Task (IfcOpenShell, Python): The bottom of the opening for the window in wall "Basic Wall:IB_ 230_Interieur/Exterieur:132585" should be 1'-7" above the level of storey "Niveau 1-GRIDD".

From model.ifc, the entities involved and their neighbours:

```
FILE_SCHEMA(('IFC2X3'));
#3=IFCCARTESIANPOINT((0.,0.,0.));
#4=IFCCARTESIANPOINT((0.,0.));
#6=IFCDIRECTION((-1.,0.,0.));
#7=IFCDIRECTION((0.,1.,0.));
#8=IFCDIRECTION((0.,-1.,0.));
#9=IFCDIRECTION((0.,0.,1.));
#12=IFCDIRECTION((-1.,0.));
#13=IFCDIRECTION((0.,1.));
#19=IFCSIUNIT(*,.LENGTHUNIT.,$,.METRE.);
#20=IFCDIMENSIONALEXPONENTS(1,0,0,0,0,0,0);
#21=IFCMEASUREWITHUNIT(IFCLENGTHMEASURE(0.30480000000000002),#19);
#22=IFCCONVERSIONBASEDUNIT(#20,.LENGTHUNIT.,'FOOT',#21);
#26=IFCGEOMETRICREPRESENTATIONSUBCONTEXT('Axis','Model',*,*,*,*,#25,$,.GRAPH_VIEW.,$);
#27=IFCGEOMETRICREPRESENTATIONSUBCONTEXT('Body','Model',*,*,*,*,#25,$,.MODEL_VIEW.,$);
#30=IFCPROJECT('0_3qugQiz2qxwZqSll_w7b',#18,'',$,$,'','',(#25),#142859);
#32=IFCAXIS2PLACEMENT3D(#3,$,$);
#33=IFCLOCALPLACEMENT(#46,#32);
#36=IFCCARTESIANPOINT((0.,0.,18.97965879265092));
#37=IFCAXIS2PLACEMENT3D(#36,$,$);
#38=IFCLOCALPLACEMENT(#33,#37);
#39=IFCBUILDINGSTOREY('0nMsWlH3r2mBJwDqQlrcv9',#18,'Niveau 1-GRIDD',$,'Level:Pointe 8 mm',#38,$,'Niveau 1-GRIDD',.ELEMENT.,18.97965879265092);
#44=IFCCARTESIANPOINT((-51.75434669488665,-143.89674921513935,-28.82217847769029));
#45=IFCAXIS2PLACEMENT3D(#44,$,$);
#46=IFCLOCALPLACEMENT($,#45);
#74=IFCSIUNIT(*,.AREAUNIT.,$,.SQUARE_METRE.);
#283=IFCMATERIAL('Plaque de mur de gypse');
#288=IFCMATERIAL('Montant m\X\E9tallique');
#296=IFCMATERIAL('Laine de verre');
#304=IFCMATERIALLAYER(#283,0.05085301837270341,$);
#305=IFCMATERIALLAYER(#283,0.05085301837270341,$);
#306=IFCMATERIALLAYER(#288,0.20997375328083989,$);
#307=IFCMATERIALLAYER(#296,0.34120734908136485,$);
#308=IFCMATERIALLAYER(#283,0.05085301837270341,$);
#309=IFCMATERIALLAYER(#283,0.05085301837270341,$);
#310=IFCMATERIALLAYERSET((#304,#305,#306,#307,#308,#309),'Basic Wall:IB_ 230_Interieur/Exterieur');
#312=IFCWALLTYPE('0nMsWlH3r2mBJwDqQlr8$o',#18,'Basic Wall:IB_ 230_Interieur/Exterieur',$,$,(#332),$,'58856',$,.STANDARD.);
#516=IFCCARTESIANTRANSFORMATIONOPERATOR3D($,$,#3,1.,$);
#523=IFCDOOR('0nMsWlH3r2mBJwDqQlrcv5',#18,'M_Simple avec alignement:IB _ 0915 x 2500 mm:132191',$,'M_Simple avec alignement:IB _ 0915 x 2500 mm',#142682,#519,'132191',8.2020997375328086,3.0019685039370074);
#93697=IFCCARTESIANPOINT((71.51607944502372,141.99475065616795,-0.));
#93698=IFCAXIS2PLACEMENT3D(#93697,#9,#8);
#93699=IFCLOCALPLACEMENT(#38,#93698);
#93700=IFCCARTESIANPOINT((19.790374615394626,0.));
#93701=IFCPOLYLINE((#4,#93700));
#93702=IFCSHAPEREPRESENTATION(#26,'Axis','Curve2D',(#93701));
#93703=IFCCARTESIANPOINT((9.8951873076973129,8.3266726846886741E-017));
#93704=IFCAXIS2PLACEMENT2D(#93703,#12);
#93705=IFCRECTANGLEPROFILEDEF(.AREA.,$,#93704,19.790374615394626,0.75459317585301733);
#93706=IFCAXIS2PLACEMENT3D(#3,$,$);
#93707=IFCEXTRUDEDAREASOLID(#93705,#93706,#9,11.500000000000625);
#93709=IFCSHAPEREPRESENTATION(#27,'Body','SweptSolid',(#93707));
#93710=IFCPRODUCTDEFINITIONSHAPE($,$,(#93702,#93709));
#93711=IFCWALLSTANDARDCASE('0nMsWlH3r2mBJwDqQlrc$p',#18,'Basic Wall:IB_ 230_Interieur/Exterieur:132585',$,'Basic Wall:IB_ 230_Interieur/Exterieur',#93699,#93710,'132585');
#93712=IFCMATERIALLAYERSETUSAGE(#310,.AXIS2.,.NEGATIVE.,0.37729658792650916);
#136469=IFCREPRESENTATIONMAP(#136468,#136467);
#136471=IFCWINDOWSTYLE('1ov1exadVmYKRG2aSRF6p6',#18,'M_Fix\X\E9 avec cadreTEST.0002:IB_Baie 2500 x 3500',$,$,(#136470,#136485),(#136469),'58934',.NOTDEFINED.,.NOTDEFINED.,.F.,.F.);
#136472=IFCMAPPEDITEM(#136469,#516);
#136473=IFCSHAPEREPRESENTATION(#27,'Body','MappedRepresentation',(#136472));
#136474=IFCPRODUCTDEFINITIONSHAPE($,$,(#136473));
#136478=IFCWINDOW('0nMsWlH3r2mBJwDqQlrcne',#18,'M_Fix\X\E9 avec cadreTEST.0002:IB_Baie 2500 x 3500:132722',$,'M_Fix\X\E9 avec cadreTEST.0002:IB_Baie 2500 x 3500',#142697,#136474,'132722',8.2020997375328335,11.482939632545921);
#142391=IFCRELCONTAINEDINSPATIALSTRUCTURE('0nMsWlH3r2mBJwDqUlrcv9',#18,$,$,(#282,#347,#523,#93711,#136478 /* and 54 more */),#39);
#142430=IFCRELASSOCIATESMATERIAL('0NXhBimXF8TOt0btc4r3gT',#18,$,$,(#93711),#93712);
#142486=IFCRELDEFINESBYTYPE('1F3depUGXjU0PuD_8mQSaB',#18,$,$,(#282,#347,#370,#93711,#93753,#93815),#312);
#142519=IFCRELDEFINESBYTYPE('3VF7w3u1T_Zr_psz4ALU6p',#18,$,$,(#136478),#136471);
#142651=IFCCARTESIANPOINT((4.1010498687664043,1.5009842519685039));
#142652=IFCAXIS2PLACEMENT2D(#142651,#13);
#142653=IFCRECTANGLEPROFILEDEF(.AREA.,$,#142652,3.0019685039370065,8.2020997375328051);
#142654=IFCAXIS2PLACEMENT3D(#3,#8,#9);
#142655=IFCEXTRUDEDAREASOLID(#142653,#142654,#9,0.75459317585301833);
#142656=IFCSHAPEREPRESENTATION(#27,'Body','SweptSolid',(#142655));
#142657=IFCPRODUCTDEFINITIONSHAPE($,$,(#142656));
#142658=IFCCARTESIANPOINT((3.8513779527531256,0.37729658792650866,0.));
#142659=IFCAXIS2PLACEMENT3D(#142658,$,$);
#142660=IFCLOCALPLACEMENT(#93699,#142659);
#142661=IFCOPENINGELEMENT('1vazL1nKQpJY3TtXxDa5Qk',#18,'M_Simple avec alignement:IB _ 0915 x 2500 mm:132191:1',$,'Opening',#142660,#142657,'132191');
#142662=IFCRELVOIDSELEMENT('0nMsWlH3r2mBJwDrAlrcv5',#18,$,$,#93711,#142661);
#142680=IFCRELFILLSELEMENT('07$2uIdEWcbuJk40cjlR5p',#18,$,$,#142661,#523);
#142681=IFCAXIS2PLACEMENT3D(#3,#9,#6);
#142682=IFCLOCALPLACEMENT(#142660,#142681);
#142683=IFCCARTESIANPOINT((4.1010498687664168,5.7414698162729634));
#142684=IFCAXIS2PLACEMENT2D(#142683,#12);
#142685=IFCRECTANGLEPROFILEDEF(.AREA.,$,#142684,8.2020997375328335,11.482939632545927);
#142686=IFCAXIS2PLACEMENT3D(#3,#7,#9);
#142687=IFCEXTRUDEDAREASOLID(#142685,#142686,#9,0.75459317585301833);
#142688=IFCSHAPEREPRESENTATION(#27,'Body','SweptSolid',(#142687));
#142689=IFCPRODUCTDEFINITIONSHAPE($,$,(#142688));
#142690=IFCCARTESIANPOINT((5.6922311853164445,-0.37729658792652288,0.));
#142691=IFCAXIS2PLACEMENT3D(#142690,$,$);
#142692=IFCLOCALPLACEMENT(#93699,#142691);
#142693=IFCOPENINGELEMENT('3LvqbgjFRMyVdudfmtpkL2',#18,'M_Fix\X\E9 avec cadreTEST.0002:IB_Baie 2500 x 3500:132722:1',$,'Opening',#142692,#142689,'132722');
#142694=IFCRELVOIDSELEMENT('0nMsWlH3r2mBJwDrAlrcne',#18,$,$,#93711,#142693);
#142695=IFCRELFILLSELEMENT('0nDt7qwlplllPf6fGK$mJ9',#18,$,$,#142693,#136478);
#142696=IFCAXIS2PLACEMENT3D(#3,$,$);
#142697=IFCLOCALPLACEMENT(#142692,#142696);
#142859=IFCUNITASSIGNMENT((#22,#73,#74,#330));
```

```python
import numpy as np
import ifcopenshell
import ifcopenshell.api.geometry
import ifcopenshell.geom
import ifcopenshell.util.element
import ifcopenshell.util.placement
import ifcopenshell.util.shape
import ifcopenshell.util.unit

model = ifcopenshell.open("model.ifc")
unit_scale = ifcopenshell.util.unit.calculate_unit_scale(model)

window = model.by_guid("0nMsWlH3r2mBJwDqQlrcne")
opening = window.FillsVoids[0].RelatingOpeningElement
storey = ifcopenshell.util.element.get_container(window, ifc_class="IfcBuildingStorey")
level = ifcopenshell.util.placement.get_local_placement(storey.ObjectPlacement)[2, 3]

# The opening's origin need not be at the sill, so measure its lowest point.
shape = ifcopenshell.geom.create_shape(ifcopenshell.geom.settings(), opening)
bottom = ifcopenshell.util.shape.get_shape_bottom_elevation(shape, shape.geometry) / unit_scale
dz = level + 19 * 0.0254 / unit_scale - bottom

shift = np.array([0.0, 0.0, dz])
# The window is placed relative to its opening, so it follows when the opening moves.
matrix = ifcopenshell.util.placement.get_local_placement(opening.ObjectPlacement)
matrix[:3, 3] += shift
ifcopenshell.api.geometry.edit_object_placement(
    model, product=opening, matrix=matrix, is_si=False, should_transform_children=True
)

print(f"moved by {dz * unit_scale:+.3f} m")

model.write("model-out.ifc")
```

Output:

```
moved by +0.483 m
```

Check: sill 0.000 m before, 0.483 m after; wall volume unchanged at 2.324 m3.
